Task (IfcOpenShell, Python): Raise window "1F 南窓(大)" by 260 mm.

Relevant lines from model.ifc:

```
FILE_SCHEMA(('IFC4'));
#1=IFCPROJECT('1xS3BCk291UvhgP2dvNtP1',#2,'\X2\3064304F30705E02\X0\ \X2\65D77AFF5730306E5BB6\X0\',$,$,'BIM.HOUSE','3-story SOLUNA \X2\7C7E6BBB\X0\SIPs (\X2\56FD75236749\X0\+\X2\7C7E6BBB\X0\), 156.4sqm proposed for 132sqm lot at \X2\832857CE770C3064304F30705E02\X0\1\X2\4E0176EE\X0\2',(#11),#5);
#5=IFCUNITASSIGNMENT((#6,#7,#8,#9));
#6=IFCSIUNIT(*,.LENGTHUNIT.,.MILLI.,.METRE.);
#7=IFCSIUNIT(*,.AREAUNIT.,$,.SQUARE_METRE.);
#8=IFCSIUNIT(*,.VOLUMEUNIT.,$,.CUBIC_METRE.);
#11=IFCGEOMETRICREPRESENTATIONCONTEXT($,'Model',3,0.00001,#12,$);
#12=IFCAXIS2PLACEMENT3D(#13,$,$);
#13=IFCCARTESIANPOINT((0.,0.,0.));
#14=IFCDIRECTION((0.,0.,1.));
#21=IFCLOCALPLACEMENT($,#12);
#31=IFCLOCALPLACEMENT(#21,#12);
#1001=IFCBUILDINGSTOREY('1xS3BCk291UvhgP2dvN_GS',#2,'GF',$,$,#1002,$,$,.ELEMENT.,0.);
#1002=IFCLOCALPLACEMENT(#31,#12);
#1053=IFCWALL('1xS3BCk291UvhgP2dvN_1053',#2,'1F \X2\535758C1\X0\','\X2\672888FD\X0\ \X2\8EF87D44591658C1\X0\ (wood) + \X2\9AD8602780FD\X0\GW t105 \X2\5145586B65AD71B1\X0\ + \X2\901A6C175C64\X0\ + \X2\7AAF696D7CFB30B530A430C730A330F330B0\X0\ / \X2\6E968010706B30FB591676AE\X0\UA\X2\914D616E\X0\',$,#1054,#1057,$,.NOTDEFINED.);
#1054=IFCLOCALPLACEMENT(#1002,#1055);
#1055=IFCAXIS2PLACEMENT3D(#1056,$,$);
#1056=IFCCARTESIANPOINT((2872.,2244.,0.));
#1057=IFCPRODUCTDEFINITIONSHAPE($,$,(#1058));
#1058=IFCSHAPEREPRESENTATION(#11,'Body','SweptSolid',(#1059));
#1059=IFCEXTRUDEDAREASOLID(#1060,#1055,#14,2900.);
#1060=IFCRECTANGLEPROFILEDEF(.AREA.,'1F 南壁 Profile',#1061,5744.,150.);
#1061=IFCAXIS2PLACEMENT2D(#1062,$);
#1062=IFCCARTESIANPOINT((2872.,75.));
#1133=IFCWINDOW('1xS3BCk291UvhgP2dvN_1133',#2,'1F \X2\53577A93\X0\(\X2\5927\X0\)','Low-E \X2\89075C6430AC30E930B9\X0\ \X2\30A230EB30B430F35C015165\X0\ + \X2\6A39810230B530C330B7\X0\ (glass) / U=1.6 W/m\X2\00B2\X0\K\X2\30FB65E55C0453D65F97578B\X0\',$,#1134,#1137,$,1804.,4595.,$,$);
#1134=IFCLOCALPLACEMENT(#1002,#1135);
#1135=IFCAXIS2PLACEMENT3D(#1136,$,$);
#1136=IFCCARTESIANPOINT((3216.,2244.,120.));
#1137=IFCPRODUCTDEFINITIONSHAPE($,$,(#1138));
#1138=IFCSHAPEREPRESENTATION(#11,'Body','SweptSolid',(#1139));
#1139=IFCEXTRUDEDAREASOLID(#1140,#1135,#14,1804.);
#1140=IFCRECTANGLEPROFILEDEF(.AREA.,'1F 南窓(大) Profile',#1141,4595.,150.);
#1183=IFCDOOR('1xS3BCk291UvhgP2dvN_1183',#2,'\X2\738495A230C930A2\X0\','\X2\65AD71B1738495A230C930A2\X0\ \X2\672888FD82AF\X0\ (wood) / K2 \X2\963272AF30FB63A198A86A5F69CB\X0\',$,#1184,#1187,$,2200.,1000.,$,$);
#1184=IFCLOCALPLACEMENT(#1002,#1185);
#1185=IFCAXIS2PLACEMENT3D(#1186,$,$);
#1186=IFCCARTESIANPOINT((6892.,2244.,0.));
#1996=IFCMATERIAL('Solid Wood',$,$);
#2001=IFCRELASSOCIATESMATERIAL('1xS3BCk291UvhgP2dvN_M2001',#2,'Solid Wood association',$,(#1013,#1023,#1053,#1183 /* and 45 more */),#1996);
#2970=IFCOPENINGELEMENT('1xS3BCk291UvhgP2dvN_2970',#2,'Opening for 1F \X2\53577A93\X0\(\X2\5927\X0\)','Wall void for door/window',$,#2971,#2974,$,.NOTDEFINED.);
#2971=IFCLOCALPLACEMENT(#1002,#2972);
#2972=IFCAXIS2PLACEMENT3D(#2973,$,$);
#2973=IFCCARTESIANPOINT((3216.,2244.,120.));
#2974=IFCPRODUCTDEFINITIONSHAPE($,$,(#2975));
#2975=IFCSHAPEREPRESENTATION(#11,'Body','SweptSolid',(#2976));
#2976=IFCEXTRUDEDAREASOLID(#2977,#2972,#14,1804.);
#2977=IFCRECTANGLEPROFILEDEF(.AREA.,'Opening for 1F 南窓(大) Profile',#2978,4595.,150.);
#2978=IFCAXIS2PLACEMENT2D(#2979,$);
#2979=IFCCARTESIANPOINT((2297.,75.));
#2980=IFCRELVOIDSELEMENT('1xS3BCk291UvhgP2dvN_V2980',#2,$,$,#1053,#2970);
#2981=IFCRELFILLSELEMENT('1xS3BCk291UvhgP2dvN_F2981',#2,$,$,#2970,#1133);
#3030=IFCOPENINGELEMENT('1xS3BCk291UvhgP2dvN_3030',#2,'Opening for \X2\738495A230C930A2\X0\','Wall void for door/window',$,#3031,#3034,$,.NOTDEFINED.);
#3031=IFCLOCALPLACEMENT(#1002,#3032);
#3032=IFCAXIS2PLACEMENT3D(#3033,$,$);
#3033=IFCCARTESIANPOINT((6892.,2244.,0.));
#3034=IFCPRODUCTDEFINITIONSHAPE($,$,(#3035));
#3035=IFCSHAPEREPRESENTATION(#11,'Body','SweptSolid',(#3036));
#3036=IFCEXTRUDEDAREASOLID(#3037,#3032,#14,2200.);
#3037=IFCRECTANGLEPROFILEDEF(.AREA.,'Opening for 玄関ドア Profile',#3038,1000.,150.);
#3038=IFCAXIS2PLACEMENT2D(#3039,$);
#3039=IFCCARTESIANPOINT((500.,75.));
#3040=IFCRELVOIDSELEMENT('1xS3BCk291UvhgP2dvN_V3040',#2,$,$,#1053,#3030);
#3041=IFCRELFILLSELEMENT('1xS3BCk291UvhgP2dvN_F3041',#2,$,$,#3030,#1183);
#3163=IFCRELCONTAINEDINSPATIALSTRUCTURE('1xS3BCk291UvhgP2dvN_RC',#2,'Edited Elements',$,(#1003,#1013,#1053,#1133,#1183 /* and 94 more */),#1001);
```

```python
import numpy as np
import ifcopenshell
import ifcopenshell.api.geometry
import ifcopenshell.util.placement
import ifcopenshell.util.unit

model = ifcopenshell.open("model.ifc")
unit_scale = ifcopenshell.util.unit.calculate_unit_scale(model)

window = model.by_id(1133)
opening = window.FillsVoids[0].RelatingOpeningElement
dz = 260.0

shift = np.array([0.0, 0.0, dz])
# The window is not placed relative to its opening, so move both.
for product in (opening, window):
    matrix = ifcopenshell.util.placement.get_local_placement(product.ObjectPlacement)
    matrix[:3, 3] += shift
    ifcopenshell.api.geometry.edit_object_placement(model, product=product, matrix=matrix, is_si=False)

print(f"moved by {dz * unit_scale:+.3f} m")

model.write("model_rev.ifc")
```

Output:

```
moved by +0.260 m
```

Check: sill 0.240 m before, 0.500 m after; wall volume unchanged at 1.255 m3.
